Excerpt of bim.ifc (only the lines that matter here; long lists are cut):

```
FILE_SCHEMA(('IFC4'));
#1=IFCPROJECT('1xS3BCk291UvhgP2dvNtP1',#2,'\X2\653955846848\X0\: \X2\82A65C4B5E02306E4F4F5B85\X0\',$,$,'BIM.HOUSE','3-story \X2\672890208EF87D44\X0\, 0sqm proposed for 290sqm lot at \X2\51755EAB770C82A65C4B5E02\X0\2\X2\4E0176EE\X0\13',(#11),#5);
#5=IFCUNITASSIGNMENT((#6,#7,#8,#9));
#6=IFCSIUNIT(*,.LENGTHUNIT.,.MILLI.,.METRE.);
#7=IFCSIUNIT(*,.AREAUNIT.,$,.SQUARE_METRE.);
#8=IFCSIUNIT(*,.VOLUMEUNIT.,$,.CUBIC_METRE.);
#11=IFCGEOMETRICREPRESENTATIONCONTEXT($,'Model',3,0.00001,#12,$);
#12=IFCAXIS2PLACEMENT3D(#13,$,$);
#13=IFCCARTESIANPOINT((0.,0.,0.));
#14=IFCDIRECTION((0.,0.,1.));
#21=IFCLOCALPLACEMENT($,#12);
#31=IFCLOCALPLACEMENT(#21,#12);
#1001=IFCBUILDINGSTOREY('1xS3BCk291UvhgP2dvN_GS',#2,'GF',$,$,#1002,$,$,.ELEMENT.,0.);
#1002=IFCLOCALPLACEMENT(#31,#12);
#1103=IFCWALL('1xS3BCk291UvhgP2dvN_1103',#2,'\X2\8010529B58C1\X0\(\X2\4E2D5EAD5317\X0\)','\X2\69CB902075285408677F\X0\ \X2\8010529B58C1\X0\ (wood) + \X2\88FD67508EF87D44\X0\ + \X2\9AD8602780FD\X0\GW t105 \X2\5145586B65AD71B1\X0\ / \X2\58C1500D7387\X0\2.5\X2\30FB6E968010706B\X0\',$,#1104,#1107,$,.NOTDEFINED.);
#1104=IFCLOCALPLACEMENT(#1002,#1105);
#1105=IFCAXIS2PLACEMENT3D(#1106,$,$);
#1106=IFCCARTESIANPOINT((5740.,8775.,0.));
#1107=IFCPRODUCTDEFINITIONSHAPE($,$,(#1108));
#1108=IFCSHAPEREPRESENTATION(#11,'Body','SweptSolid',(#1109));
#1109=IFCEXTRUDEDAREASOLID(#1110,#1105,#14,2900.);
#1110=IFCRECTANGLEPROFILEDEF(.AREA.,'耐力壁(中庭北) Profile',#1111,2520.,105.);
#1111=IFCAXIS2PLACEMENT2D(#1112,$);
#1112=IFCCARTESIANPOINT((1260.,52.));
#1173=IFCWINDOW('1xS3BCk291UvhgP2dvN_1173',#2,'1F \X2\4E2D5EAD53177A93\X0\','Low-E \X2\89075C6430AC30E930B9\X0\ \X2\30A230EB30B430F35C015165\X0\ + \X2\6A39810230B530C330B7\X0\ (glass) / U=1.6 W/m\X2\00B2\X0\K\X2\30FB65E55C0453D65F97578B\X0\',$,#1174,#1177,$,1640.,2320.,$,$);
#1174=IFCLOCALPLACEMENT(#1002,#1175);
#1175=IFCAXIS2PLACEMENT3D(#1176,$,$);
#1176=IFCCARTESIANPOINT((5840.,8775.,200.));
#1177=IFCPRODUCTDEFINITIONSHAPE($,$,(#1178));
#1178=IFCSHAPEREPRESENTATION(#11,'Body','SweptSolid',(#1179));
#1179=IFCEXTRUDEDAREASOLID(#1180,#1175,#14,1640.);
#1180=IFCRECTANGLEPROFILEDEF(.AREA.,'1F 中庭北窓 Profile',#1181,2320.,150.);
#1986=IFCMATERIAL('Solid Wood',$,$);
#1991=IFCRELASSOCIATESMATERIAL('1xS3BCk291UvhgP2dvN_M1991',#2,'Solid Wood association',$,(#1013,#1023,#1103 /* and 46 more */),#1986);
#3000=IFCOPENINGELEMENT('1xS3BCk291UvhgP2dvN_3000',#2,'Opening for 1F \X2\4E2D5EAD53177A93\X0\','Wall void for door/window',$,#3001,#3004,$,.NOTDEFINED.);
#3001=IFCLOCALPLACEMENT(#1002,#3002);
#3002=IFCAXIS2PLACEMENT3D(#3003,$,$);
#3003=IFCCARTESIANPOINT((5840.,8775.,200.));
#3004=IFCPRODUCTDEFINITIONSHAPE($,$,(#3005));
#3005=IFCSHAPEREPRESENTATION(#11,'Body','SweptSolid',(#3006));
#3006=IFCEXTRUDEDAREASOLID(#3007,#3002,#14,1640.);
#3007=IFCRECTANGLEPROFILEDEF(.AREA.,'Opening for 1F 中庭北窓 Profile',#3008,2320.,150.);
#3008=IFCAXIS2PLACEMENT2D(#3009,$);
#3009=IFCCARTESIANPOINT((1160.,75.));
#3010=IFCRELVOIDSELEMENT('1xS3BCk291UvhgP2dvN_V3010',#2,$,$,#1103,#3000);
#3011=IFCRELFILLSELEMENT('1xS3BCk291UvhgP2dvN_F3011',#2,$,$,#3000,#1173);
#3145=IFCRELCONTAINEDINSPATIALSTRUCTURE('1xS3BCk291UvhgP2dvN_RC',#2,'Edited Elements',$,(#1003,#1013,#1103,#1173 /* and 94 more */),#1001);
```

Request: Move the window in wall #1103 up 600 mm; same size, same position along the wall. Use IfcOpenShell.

```python
import numpy as np
import ifcopenshell
import ifcopenshell.api.geometry
import ifcopenshell.util.placement
import ifcopenshell.util.unit

model = ifcopenshell.open("bim.ifc")
unit_scale = ifcopenshell.util.unit.calculate_unit_scale(model)

window = model.by_guid("1xS3BCk291UvhgP2dvN_1173")
opening = window.FillsVoids[0].RelatingOpeningElement
dz = 0.6 / unit_scale

shift = np.array([0.0, 0.0, dz])
# The window is not placed relative to its opening, so move both.
for product in (opening, window):
    matrix = ifcopenshell.util.placement.get_local_placement(product.ObjectPlacement)
    matrix[:3, 3] += shift
    ifcopenshell.api.geometry.edit_object_placement(model, product=product, matrix=matrix, is_si=False)

print(f"moved by {dz * unit_scale:+.3f} m")

model.write("bim_updated.ifc")
```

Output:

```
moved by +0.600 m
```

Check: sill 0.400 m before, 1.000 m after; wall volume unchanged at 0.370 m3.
